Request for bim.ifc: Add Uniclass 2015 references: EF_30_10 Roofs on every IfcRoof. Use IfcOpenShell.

First a look at what the model holds.

```python
import ifcopenshell

model = ifcopenshell.open("bim.ifc")
print(model.schema)
print("classifications:", [c.Name for c in model.by_type("IfcClassification")])
for ifc_class in ("IfcDoor", "IfcRoof", "IfcStair", "IfcWall", "IfcWindow"):
    print(ifc_class, len(model.by_type(ifc_class)))
```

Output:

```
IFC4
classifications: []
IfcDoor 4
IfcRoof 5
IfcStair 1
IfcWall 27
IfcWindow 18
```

```python
import ifcopenshell
import ifcopenshell.api.classification

model = ifcopenshell.open("bim.ifc")

system = ifcopenshell.api.classification.add_classification(model, classification="Uniclass 2015")

codes = {
    "IfcRoof": ("EF_30_10", "Roofs"),
}
for ifc_class, (code, name) in codes.items():
    products = model.by_type(ifc_class)
    ifcopenshell.api.classification.add_reference(
        model, products=products, classification=system, identification=code, name=name
    )
    print(code, len(products))

model.write("bim-out.ifc")
```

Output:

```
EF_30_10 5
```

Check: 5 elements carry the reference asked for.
